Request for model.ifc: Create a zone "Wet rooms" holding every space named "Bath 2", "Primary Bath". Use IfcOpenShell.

First a look at what the model holds.

```python
import ifcopenshell

model = ifcopenshell.open("model.ifc")
print(model.schema)
seen = {}
for space in model.by_type("IfcSpace"):
    seen[space.LongName] = seen.get(space.LongName, 0) + 1
for name, count in sorted(seen.items(), key=str):
    print(count, "x", name)
print("zones:", [z.Name for z in model.by_type("IfcZone")][:20])
```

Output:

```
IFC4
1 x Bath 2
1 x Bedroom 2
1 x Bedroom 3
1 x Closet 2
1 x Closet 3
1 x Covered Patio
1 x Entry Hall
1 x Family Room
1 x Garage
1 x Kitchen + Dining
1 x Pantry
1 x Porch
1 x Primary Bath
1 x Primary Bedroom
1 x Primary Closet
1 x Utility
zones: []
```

```python
import ifcopenshell
import ifcopenshell.api.group
import ifcopenshell.api.root

model = ifcopenshell.open("model.ifc")

names = {"Bath 2", "Primary Bath"}
spaces = [s for s in model.by_type("IfcSpace") if s.LongName in names]

zone = ifcopenshell.api.root.create_entity(model, ifc_class="IfcZone", name="Wet rooms")
ifcopenshell.api.group.assign_group(model, products=spaces, group=zone)
print(len(spaces), "spaces in", zone.Name)

model.write("model_v2.ifc")
```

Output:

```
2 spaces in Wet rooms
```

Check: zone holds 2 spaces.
